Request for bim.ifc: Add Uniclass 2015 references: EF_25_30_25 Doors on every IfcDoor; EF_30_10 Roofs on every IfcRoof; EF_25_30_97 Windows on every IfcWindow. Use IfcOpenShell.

First a look at what the model holds.

```python
import ifcopenshell

model = ifcopenshell.open("bim.ifc")
print(model.schema)
print("classifications:", [c.Name for c in model.by_type("IfcClassification")])
for ifc_class in ("IfcDoor", "IfcRoof", "IfcStair", "IfcWall", "IfcWindow"):
    print(ifc_class, len(model.by_type(ifc_class)))
```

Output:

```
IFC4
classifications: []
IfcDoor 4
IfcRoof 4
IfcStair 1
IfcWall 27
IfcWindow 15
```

```python
import ifcopenshell
import ifcopenshell.api.classification

model = ifcopenshell.open("bim.ifc")

system = ifcopenshell.api.classification.add_classification(model, classification="Uniclass 2015")

codes = {
    "IfcDoor": ("EF_25_30_25", "Doors"),
    "IfcRoof": ("EF_30_10", "Roofs"),
    "IfcWindow": ("EF_25_30_97", "Windows"),
}
for ifc_class, (code, name) in codes.items():
    products = model.by_type(ifc_class)
    ifcopenshell.api.classification.add_reference(
        model, products=products, classification=system, identification=code, name=name
    )
    print(code, len(products))

model.write("bim_edited.ifc")
```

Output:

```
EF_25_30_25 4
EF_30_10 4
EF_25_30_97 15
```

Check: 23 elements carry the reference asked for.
